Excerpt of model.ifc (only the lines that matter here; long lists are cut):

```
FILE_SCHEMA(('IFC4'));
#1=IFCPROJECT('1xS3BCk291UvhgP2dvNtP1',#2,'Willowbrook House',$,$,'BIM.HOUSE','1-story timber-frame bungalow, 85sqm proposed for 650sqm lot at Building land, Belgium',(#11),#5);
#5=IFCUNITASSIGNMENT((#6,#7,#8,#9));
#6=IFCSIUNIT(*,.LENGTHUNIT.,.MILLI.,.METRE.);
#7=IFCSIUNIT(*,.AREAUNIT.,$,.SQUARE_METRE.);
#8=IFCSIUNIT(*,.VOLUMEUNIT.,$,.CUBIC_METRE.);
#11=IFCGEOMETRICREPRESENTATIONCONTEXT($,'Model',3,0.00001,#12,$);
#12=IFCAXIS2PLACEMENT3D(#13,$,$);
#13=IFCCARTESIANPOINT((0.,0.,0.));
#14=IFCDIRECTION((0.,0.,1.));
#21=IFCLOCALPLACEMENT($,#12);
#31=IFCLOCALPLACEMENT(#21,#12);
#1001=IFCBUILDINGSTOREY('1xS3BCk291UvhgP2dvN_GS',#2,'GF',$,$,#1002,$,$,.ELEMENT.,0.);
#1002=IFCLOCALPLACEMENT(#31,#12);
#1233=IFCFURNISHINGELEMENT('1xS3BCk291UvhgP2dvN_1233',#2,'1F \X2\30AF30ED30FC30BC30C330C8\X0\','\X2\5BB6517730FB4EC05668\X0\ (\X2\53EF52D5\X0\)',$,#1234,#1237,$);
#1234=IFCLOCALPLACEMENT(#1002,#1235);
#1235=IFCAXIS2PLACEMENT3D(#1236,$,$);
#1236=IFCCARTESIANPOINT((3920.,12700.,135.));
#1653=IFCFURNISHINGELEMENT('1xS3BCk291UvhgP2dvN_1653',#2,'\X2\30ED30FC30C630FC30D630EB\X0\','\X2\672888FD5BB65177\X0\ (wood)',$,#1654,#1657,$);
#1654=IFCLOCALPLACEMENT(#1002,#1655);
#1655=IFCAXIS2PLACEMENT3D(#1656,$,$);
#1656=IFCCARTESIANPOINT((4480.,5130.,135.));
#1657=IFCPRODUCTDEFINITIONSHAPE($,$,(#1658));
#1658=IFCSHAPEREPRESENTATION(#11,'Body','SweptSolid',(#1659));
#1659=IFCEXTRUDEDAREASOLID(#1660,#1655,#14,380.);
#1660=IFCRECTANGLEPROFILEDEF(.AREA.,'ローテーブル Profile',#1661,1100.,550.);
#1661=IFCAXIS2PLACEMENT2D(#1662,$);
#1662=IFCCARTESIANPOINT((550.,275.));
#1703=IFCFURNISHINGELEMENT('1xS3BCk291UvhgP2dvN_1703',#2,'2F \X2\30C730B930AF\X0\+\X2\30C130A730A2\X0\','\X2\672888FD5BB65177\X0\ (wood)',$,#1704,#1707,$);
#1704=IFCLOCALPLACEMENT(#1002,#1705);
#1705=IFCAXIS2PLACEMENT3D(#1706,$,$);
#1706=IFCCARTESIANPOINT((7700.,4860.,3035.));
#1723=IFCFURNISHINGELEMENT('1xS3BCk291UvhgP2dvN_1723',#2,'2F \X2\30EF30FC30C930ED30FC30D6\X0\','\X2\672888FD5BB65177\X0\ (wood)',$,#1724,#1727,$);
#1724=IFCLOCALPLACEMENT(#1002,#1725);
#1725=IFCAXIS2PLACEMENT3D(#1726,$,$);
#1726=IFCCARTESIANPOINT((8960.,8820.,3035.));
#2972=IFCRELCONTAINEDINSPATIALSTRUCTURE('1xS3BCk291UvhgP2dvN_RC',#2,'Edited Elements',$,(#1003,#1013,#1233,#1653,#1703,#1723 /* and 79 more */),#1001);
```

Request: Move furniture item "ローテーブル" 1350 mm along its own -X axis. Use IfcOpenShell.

```python
import ifcopenshell
import ifcopenshell.api.geometry
import ifcopenshell.util.placement
import ifcopenshell.util.unit

model = ifcopenshell.open("model.ifc")
unit_scale = ifcopenshell.util.unit.calculate_unit_scale(model)

item = model.by_guid("1xS3BCk291UvhgP2dvN_1653")
matrix = ifcopenshell.util.placement.get_local_placement(item.ObjectPlacement)
matrix[:3, 3] -= matrix[:3, 0] * 1.35 / unit_scale
ifcopenshell.api.geometry.edit_object_placement(model, product=item, matrix=matrix, is_si=False)

print(ifcopenshell.util.placement.get_local_placement(item.ObjectPlacement).round(3) + 0.0)

model.write("model-out.ifc")
```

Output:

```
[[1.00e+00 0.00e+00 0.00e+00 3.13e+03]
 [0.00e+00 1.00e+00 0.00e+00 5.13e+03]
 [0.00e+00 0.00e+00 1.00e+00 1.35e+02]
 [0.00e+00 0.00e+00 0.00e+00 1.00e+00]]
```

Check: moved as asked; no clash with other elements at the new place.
